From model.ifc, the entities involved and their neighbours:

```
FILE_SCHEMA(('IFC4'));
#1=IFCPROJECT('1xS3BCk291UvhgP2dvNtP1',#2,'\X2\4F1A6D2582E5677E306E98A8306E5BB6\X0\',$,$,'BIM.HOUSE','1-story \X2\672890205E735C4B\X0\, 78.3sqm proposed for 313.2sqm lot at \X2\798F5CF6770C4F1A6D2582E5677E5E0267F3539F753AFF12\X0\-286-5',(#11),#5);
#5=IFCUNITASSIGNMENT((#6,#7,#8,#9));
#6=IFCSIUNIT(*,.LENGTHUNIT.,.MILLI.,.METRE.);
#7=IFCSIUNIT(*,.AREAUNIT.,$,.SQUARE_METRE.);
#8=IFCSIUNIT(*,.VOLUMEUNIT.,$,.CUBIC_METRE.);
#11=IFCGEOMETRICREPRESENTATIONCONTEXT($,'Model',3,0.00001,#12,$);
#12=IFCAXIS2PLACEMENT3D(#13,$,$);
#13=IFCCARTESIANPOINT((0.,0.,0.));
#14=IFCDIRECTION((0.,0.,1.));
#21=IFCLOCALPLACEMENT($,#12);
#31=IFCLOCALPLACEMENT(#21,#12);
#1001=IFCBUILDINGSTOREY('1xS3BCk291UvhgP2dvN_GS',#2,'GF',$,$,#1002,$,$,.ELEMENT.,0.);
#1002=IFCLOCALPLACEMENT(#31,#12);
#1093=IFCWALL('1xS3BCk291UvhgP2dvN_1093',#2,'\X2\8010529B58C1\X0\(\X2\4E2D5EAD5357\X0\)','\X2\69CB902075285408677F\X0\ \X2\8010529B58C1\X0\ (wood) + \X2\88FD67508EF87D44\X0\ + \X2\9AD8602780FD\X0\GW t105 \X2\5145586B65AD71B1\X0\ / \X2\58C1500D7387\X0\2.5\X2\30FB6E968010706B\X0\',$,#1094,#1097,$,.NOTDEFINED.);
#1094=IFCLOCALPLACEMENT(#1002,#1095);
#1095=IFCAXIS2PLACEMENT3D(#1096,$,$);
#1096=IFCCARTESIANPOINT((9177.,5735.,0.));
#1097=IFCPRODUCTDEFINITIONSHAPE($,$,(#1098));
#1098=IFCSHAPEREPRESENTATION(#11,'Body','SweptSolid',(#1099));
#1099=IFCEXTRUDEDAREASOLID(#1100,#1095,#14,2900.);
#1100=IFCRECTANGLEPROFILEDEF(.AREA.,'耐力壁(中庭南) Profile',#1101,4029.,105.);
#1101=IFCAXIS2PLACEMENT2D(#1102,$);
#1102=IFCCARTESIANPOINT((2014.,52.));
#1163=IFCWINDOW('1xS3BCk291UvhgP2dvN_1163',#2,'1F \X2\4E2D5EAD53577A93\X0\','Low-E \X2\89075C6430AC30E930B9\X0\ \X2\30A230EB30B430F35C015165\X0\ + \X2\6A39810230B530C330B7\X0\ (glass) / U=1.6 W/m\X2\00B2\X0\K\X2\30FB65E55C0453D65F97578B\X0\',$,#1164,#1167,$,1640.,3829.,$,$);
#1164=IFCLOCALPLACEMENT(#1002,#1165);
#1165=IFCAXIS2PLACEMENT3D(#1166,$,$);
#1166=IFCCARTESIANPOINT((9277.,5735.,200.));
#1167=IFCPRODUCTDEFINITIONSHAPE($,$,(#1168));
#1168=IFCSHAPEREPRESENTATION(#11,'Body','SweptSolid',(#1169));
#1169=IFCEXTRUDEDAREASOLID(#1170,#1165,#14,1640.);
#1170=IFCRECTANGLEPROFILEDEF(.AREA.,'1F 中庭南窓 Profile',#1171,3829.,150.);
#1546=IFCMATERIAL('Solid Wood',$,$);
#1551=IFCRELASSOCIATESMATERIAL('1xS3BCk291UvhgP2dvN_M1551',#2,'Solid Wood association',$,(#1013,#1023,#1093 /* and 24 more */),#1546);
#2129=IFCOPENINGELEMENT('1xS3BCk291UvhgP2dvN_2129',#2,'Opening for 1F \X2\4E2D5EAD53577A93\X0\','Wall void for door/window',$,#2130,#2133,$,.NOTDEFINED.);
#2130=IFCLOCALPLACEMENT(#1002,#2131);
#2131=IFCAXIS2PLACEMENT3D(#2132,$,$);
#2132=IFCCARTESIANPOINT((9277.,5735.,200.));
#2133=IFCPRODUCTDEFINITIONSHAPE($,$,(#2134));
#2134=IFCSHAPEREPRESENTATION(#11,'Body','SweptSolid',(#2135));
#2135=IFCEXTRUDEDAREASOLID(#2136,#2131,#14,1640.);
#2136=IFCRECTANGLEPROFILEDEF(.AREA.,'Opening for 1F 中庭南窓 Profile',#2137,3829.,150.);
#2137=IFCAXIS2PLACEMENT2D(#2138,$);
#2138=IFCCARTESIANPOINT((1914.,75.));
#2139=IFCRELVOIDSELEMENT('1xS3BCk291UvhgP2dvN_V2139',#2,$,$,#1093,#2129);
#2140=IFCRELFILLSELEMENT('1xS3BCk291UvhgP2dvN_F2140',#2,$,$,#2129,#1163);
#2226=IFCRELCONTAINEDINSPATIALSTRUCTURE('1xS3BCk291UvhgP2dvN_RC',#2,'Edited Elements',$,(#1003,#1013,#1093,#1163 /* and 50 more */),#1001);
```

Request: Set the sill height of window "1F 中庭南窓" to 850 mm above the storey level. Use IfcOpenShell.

```python
import numpy as np
import ifcopenshell
import ifcopenshell.api.geometry
import ifcopenshell.geom
import ifcopenshell.util.element
import ifcopenshell.util.placement
import ifcopenshell.util.shape
import ifcopenshell.util.unit

model = ifcopenshell.open("model.ifc")
unit_scale = ifcopenshell.util.unit.calculate_unit_scale(model)

window = model.by_guid("1xS3BCk291UvhgP2dvN_1163")
opening = window.FillsVoids[0].RelatingOpeningElement
storey = ifcopenshell.util.element.get_container(window, ifc_class="IfcBuildingStorey")
level = ifcopenshell.util.placement.get_local_placement(storey.ObjectPlacement)[2, 3]

# The opening's origin need not be at the sill, so measure its lowest point.
shape = ifcopenshell.geom.create_shape(ifcopenshell.geom.settings(), opening)
bottom = ifcopenshell.util.shape.get_shape_bottom_elevation(shape, shape.geometry) / unit_scale
dz = level + 0.85 / unit_scale - bottom

shift = np.array([0.0, 0.0, dz])
# The window is not placed relative to its opening, so move both.
for product in (opening, window):
    matrix = ifcopenshell.util.placement.get_local_placement(product.ObjectPlacement)
    matrix[:3, 3] += shift
    ifcopenshell.api.geometry.edit_object_placement(model, product=product, matrix=matrix, is_si=False)

print(f"moved by {dz * unit_scale:+.3f} m")

model.write("model-out.ifc")
```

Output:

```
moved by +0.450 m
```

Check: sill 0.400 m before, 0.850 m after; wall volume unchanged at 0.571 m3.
